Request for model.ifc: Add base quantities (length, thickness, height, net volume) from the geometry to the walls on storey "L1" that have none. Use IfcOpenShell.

First a look at what the model holds.

```python
import ifcopenshell
import ifcopenshell.util.element
import ifcopenshell.util.unit

model = ifcopenshell.open("model.ifc")
print(model.schema)
for unit_type in ("LENGTHUNIT", "AREAUNIT", "VOLUMEUNIT"):
    print(unit_type, ifcopenshell.util.unit.calculate_unit_scale(model, unit_type))
storey = next(s for s in model.by_type("IfcBuildingStorey") if s.Name == "L1")
walls = [e for e in ifcopenshell.util.element.get_decomposition(storey) if e.is_a("IfcWall")]
for e in sorted(walls, key=lambda e: e.id()):
    print(e.id(), e.is_a(), e.Name, list(ifcopenshell.util.element.get_psets(e, qtos_only=True)), sep=" | ")
```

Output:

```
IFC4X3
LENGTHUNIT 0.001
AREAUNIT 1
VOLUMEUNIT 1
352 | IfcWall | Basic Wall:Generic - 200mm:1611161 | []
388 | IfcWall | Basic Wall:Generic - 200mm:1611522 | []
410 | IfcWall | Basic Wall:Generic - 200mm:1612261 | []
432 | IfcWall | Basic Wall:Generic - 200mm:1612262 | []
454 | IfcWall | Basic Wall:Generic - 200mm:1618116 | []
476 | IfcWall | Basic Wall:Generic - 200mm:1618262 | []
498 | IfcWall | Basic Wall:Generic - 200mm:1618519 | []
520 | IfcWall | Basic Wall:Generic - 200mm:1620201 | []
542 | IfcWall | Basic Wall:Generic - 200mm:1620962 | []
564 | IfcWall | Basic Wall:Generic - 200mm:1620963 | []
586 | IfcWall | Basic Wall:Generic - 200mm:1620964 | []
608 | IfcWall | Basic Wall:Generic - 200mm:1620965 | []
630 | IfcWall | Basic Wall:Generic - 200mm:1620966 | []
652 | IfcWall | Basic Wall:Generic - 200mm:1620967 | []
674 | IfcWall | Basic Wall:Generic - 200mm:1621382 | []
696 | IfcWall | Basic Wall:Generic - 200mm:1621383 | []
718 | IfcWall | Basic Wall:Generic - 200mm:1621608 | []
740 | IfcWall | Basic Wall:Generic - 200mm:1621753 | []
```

```python
import ifcopenshell
import ifcopenshell.api.pset
import ifcopenshell.geom
import ifcopenshell.util.element
import ifcopenshell.util.shape
import ifcopenshell.util.unit

model = ifcopenshell.open("model.ifc")
unit_scale = ifcopenshell.util.unit.calculate_unit_scale(model)
volume_scale = ifcopenshell.util.unit.calculate_unit_scale(model, "VOLUMEUNIT")
settings = ifcopenshell.geom.settings()

storey = next(s for s in model.by_type("IfcBuildingStorey") if s.Name == "L1")
walls = [e for e in ifcopenshell.util.element.get_decomposition(storey) if e.is_a("IfcWall")]

for e in sorted(walls, key=lambda e: e.id()):
    if ifcopenshell.util.element.get_psets(e, qtos_only=True, should_inherit=False):
        continue
    # Geometry comes back in metres, in the element's own axes.
    shape = ifcopenshell.geom.create_shape(settings, e)
    values = {
        "Length": ifcopenshell.util.shape.get_x(shape.geometry) / unit_scale,
        "Width": ifcopenshell.util.shape.get_y(shape.geometry) / unit_scale,
        "Height": ifcopenshell.util.shape.get_z(shape.geometry) / unit_scale,
        "NetVolume": ifcopenshell.util.shape.get_volume(shape.geometry) / volume_scale,
    }
    qto = ifcopenshell.api.pset.add_qto(model, product=e, name="Qto_WallBaseQuantities")
    ifcopenshell.api.pset.edit_qto(model, qto=qto, properties=values)
    print(e.id(), {k: round(v, 3) for k, v in values.items()})

model.write("model_updated.ifc")
```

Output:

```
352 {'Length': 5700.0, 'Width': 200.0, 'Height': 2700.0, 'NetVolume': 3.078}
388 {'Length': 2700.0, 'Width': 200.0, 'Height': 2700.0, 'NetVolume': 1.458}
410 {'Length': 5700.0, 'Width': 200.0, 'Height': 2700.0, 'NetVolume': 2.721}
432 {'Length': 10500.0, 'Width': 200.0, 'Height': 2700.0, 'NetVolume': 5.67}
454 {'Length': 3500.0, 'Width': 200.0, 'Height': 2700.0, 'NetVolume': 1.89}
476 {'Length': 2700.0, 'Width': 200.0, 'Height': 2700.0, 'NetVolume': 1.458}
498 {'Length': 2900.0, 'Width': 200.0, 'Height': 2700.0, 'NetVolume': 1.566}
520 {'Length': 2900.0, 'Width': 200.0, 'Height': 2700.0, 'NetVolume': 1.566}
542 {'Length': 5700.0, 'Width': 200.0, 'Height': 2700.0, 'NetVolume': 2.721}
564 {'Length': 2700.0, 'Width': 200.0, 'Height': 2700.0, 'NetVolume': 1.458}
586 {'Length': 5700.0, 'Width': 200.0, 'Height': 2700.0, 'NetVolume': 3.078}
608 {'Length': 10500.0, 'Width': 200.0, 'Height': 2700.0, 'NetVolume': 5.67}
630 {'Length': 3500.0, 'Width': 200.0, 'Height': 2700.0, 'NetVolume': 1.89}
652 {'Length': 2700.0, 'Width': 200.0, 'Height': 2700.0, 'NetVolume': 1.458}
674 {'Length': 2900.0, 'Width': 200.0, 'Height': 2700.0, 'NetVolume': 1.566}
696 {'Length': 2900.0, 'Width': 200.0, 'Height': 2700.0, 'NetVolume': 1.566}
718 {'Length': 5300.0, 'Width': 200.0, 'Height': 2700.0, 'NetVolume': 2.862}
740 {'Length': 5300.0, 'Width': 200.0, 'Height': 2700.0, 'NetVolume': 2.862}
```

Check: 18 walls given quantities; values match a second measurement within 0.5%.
